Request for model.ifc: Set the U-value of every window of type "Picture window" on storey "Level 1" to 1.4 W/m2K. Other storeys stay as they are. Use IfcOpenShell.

First a look at what the model holds.

```python
import ifcopenshell
import ifcopenshell.util.element

model = ifcopenshell.open("model.ifc")
print(model.schema)
storey = next(s for s in model.by_type("IfcBuildingStorey") if s.Name == "Level 1")
windows = [e for e in ifcopenshell.util.element.get_decomposition(storey) if e.is_a("IfcWindow")]
seen = {}
for e in windows:
    element_type = ifcopenshell.util.element.get_type(e)
    key = (element_type.Name if element_type != e and element_type else None, ifcopenshell.util.element.get_pset(e, "Pset_WindowCommon", "ThermalTransmittance"))
    seen[key] = seen.get(key, 0) + 1
for (name, value), count in sorted(seen.items(), key=str):
    print(count, "x", name, "|", value)
```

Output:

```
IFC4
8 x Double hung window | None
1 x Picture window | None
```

```python
import ifcopenshell
import ifcopenshell.api.pset
import ifcopenshell.util.element

model = ifcopenshell.open("model.ifc")

storey = next(s for s in model.by_type("IfcBuildingStorey") if s.Name == "Level 1")
windows = [e for e in ifcopenshell.util.element.get_decomposition(storey) if e.is_a("IfcWindow")]

count = 0
for e in windows:
    element_type = ifcopenshell.util.element.get_type(e)
    if element_type in (None, e) or element_type.Name != "Picture window":
        continue
    # add_pset returns the element's existing set when there is one.
    pset = ifcopenshell.api.pset.add_pset(model, product=e, name="Pset_WindowCommon")
    ifcopenshell.api.pset.edit_pset(model, pset=pset, properties={"ThermalTransmittance": 1.4})
    count += 1

print(count, "windows updated")

model.write("model_v2.ifc")
```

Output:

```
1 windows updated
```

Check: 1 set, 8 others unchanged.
